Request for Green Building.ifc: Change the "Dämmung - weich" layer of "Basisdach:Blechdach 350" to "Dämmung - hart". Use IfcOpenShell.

First a look at what the model holds.

```python
import ifcopenshell
import ifcopenshell.util.element

model = ifcopenshell.open("Green Building.ifc")
print(model.schema)
for layer_set in model.by_type("IfcMaterialLayerSet"):
    if layer_set.LayerSetName == "Basisdach:Blechdach 350":
        for layer in layer_set.MaterialLayers:
            print(layer.id(), layer.Material and layer.Material.Name, layer.LayerThickness, sep=" | ")
        print(len(ifcopenshell.util.element.get_elements_by_material(model, layer_set)), "elements and types use it")
print(sorted(m.Name for m in model.by_type("IfcMaterial") if m.Name)[:60])
```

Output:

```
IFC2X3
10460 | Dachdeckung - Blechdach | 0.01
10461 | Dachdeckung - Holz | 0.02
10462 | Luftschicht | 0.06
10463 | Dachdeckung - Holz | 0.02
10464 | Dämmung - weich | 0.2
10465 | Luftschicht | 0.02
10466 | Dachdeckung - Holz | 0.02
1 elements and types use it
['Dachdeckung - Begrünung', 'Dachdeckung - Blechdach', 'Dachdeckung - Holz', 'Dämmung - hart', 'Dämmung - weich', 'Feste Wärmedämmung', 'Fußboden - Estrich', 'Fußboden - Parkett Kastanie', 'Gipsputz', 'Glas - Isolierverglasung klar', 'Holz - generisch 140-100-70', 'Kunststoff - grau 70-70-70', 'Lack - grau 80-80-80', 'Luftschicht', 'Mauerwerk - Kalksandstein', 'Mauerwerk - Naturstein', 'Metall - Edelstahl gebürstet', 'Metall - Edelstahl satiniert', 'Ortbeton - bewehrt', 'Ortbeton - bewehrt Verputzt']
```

```python
import ifcopenshell
import ifcopenshell.api.material

model = ifcopenshell.open("Green Building.ifc")

layer_set = next(s for s in model.by_type("IfcMaterialLayerSet") if s.LayerSetName == "Basisdach:Blechdach 350")
layer = next(l for l in layer_set.MaterialLayers if l.Material and l.Material.Name == "Dämmung - weich")
material = next(m for m in model.by_type("IfcMaterial") if m.Name == "Dämmung - hart")

# Point this one layer at the other material; renaming the old one would change it everywhere.
ifcopenshell.api.material.edit_layer(model, layer=layer, attributes={}, material=material)

print([l.Material.Name if l.Material else None for l in layer_set.MaterialLayers])

model.write("Green Building-out.ifc")
```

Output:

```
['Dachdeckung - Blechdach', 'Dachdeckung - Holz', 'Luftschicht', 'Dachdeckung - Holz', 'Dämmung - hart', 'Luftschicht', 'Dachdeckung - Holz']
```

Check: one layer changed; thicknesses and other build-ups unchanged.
